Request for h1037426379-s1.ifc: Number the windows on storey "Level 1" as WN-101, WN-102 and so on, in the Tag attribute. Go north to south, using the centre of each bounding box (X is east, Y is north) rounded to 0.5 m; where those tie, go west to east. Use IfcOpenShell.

First a look at what the model holds.

```python
import ifcopenshell
import ifcopenshell.util.element
import ifcopenshell.util.placement

model = ifcopenshell.open("h1037426379-s1.ifc")
print(model.schema)
storey = next(s for s in model.by_type("IfcBuildingStorey") if s.Name == "Level 1")
windows = [e for e in ifcopenshell.util.element.get_decomposition(storey) if e.is_a("IfcWindow")]
for e in sorted(windows, key=lambda e: e.id()):
    origin = ifcopenshell.util.placement.get_local_placement(e.ObjectPlacement)[:3, 3]
    print(e.id(), e.Tag, e.Name, origin.round(2) + 0.0, sep=" | ")
```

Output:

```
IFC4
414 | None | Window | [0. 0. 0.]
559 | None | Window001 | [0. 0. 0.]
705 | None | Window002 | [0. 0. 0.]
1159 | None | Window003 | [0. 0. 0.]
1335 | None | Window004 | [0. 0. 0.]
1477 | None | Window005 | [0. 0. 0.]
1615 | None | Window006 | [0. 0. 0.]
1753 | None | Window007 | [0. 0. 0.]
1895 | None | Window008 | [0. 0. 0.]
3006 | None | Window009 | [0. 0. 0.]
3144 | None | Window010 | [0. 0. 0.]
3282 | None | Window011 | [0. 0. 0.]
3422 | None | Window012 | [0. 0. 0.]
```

```python
import ifcopenshell
import ifcopenshell.geom
import ifcopenshell.util.element
import ifcopenshell.util.shape

model = ifcopenshell.open("h1037426379-s1.ifc")
settings = ifcopenshell.geom.settings()
settings.set("use-world-coords", True)


def centre(element):
    shape = ifcopenshell.geom.create_shape(settings, element)
    return ifcopenshell.util.shape.get_bbox_centroid(shape.geometry)


storey = next(s for s in model.by_type("IfcBuildingStorey") if s.Name == "Level 1")
windows = [e for e in ifcopenshell.util.element.get_decomposition(storey) if e.is_a("IfcWindow")]

# Insertion points can sit at a corner or the storey origin, so sort by the geometry (in metres).
centres = {e: centre(e) for e in windows}
windows.sort(key=lambda e: (-round(centres[e][1] / 0.5), centres[e][0]))

for i, e in enumerate(windows, start=1):
    number = f"WN-1{i:02d}"
    e.Tag = number
    print(e.id(), number)

model.write("h1037426379-s1_v2.ifc")
```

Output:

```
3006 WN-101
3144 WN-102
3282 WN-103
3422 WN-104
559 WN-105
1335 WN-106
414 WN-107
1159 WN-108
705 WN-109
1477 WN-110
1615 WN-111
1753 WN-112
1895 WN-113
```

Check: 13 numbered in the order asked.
